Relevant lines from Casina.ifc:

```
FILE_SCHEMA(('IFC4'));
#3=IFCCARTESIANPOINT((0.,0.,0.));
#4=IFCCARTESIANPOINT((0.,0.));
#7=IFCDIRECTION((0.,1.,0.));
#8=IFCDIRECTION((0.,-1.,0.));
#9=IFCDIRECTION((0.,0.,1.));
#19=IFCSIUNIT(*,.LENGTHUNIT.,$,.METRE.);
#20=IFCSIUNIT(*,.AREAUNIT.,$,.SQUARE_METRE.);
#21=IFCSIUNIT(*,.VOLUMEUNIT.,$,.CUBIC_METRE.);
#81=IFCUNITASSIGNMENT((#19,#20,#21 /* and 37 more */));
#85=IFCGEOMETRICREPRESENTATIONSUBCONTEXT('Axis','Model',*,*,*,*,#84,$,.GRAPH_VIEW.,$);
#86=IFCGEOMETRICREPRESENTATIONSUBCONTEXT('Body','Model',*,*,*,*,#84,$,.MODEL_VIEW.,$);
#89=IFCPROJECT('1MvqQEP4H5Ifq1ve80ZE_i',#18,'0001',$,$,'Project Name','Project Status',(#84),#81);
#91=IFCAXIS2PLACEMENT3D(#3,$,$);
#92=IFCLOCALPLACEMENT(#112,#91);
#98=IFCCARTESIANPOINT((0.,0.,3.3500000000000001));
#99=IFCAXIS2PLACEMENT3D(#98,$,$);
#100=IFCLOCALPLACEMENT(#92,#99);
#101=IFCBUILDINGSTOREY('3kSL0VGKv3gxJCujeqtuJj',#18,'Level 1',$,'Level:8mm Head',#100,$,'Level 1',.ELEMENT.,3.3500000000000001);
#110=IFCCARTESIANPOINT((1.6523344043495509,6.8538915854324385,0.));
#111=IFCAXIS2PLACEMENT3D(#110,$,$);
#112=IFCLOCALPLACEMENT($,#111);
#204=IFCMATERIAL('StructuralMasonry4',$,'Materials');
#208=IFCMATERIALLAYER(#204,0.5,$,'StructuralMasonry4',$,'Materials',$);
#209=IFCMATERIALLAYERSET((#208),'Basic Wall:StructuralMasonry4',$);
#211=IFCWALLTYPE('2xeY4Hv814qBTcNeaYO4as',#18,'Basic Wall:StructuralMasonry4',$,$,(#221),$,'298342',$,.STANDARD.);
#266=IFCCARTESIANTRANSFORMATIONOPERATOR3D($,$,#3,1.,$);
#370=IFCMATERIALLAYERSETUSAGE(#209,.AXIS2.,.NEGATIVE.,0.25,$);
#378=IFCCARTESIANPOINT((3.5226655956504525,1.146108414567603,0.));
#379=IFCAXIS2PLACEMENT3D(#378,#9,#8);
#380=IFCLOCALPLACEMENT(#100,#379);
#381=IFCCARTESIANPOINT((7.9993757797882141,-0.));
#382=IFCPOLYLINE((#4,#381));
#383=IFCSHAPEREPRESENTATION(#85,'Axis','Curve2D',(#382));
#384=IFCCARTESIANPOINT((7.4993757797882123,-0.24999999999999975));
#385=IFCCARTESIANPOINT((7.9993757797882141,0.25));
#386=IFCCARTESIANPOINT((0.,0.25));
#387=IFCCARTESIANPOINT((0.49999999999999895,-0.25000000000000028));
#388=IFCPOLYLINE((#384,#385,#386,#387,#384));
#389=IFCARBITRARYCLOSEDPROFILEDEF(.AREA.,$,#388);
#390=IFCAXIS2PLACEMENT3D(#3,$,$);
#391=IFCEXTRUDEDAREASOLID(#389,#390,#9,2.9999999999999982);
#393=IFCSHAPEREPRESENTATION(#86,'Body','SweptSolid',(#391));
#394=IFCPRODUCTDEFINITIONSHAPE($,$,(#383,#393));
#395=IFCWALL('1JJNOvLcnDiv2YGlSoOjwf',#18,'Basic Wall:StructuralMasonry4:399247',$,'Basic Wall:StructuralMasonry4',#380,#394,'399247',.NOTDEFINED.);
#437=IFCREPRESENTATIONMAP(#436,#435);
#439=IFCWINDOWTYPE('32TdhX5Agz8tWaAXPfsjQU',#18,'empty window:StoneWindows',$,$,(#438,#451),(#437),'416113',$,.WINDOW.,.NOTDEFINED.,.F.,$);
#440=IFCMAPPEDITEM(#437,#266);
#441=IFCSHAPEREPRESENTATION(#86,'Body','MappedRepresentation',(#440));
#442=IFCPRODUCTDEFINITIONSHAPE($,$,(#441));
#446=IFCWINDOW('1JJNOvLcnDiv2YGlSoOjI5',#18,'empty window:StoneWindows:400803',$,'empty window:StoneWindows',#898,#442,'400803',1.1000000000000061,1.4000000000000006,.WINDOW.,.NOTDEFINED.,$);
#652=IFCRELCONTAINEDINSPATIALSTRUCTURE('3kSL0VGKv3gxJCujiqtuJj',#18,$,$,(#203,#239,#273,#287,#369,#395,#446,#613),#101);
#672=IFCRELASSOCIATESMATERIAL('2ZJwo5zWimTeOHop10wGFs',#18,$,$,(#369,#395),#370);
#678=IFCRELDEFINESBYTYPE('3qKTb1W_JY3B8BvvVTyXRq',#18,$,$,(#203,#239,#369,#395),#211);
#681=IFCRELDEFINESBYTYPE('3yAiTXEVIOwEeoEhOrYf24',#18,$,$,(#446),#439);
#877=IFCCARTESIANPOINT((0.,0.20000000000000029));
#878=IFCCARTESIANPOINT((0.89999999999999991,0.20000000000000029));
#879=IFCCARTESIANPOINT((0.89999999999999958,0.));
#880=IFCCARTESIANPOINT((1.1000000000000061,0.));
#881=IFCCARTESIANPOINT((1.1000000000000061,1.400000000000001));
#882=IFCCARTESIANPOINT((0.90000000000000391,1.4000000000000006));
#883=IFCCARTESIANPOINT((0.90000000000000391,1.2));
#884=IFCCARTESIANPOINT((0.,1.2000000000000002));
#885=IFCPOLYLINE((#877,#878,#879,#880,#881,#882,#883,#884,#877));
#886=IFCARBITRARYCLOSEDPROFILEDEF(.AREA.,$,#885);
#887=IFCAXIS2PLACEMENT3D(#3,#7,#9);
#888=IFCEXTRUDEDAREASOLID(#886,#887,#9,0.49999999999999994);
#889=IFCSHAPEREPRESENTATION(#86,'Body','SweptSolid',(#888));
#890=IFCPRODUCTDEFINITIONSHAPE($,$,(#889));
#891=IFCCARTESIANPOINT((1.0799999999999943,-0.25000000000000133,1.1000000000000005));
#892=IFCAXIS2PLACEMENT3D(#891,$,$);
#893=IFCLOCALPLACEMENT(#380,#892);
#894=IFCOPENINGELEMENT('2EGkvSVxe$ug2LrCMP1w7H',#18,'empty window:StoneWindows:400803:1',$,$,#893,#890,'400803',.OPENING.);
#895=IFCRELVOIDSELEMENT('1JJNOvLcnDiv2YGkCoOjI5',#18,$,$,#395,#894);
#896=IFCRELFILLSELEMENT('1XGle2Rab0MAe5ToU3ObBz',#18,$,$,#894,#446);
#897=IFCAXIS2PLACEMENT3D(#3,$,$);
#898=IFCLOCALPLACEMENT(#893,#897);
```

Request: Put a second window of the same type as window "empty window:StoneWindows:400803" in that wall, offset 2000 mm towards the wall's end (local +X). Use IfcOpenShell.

```python
import ifcopenshell
import ifcopenshell.api.feature
import ifcopenshell.api.geometry
import ifcopenshell.api.root
import ifcopenshell.geom
import ifcopenshell.util.element
import ifcopenshell.util.placement
import ifcopenshell.util.shape

model = ifcopenshell.open("Casina.ifc")
settings = ifcopenshell.geom.settings()


def volume(element):
    """Net volume in cubic metres, openings subtracted."""
    shape = ifcopenshell.geom.create_shape(settings, element)
    return ifcopenshell.util.shape.get_volume(shape.geometry)


def reuse_history(source, copy):
    """copy_class also copies each property set's owner history, people and application; keep the originals."""
    for rel in copy.IsDefinedBy:
        if rel.is_a("IfcRelDefinesByProperties") and (history := rel.RelatingPropertyDefinition.OwnerHistory):
            rel.RelatingPropertyDefinition.OwnerHistory = source.OwnerHistory
            ifcopenshell.util.element.remove_deep2(model, history)


window = model.by_guid("1JJNOvLcnDiv2YGlSoOjI5")
opening = window.FillsVoids[0].RelatingOpeningElement
wall = opening.VoidsElements[0].RelatingBuildingElement
before = volume(wall)
shift = ifcopenshell.util.placement.get_local_placement(wall.ObjectPlacement)[:3, 0] * 2.0

# copy_class copies the void relationship, type, container and properties, but no geometry.
new_opening = ifcopenshell.api.root.copy_class(model, product=opening)
new_opening.Representation = ifcopenshell.util.element.copy_deep(
    model, opening.Representation, exclude=["IfcGeometricRepresentationContext", "IfcRepresentationMap"]
)
new_opening.Name = "empty window:StoneWindows"
new_opening.Tag = None
new_window = ifcopenshell.api.root.copy_class(model, product=window)
new_window.Representation = ifcopenshell.util.element.copy_deep(
    model, window.Representation, exclude=["IfcGeometricRepresentationContext", "IfcRepresentationMap"]
)
new_window.Name = "empty window:StoneWindows"
new_window.Tag = None
reuse_history(window, new_window)
ifcopenshell.api.feature.add_filling(model, opening=new_opening, element=new_window)

for old, new in ((opening, new_opening), (window, new_window)):
    matrix = ifcopenshell.util.placement.get_local_placement(old.ObjectPlacement)
    matrix[:3, 3] += shift
    ifcopenshell.api.geometry.edit_object_placement(model, product=new, matrix=matrix, is_si=False)

after = volume(wall)

print(f"wall volume {before:.3f} -> {after:.3f} m3")

model.write("Casina_v2.ifc")
```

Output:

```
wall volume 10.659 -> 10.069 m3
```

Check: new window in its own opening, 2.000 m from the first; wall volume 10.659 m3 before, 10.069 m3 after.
